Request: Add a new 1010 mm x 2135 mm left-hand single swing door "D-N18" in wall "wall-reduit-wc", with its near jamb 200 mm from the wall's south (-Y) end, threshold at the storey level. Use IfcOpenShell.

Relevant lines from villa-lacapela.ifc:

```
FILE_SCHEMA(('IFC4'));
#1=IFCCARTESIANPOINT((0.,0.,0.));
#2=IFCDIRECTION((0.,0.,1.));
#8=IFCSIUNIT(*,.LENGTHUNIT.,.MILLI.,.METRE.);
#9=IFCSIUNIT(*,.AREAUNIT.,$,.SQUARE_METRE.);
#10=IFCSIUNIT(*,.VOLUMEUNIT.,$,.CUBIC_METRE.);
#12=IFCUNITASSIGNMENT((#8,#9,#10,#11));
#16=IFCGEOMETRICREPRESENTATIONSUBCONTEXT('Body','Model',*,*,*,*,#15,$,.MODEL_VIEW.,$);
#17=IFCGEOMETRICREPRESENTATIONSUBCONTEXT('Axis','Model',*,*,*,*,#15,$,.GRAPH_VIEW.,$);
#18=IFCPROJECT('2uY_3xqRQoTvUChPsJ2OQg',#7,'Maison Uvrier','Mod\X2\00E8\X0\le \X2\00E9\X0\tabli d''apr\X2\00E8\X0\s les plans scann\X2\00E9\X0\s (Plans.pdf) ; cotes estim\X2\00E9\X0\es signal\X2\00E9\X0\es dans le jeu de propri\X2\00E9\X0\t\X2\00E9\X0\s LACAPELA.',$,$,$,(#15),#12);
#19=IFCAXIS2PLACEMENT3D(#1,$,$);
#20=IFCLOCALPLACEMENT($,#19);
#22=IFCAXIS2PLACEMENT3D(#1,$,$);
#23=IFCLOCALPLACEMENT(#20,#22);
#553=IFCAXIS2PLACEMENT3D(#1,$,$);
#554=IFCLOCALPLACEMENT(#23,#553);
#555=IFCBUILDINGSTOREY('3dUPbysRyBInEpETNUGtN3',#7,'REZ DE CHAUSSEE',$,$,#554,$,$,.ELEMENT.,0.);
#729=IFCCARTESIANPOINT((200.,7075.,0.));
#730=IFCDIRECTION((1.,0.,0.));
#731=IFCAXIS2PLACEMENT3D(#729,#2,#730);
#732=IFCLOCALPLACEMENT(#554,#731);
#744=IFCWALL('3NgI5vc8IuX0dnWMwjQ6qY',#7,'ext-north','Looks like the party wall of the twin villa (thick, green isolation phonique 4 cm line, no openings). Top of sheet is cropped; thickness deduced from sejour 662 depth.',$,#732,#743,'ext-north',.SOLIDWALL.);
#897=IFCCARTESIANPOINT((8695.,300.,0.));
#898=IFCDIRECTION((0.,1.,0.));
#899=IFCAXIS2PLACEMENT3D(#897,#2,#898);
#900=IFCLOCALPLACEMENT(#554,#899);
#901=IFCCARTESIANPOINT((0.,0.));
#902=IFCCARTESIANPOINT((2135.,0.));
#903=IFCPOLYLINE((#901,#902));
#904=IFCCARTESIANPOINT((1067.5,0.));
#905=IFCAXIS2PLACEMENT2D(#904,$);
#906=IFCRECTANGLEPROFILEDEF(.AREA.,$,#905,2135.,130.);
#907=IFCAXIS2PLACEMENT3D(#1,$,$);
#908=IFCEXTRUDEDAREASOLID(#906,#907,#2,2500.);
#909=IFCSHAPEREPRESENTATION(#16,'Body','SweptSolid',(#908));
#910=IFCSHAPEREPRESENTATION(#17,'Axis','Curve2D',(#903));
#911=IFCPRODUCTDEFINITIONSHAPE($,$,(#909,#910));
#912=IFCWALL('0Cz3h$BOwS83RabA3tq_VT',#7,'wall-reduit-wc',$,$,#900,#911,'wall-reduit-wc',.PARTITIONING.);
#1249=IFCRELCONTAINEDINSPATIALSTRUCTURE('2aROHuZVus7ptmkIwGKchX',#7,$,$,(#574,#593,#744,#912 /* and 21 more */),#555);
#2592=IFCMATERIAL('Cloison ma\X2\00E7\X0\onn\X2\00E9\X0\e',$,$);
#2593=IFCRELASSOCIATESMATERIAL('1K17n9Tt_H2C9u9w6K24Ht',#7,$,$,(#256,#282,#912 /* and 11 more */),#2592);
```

```python
import numpy as np
import ifcopenshell
import ifcopenshell.api.feature
import ifcopenshell.api.geometry
import ifcopenshell.api.root
import ifcopenshell.api.spatial
import ifcopenshell.geom
import ifcopenshell.util.element
import ifcopenshell.util.placement
import ifcopenshell.util.representation
import ifcopenshell.util.shape
import ifcopenshell.util.unit

model = ifcopenshell.open("villa-lacapela.ifc")
unit_scale = ifcopenshell.util.unit.calculate_unit_scale(model)
settings = ifcopenshell.geom.settings()


def volume(element):
    """Net volume in cubic metres, openings subtracted."""
    shape = ifcopenshell.geom.create_shape(settings, element)
    return ifcopenshell.util.shape.get_volume(shape.geometry)


wall = model.by_id(912)
storey = ifcopenshell.util.element.get_container(wall, ifc_class="IfcBuildingStorey")
context = ifcopenshell.util.representation.get_context(model, "Model", "Body", "MODEL_VIEW")
before = volume(wall)

width, height, from_end, sill = 1.01, 2.135, 0.2, 0.0  # metres

# The wall runs along its own X axis, and the end named is its -X end.
wall_shape = ifcopenshell.geom.create_shape(settings, wall)
x, y, z = ifcopenshell.util.shape.get_vertices(wall_shape.geometry).T
start = x.min() + from_end
face, thickness = float(y.min()), float(y.max() - y.min())
wall_matrix = ifcopenshell.util.placement.get_local_placement(wall.ObjectPlacement)
level = ifcopenshell.util.placement.get_local_placement(storey.ObjectPlacement)[2, 3]


def in_wall(x, y):
    """Placement at x, y metres in the wall's axes, at sill height."""
    matrix = wall_matrix.copy()
    matrix[:, 3] = wall_matrix @ np.array([x / unit_scale, y / unit_scale, 0.0, 1.0])
    matrix[2, 3] = level + sill / unit_scale
    return matrix


# Opening: a box that overshoots both wall faces by 50 mm.
opening = ifcopenshell.api.root.create_entity(model, ifc_class="IfcOpeningElement", predefined_type="OPENING")
box = ifcopenshell.api.geometry.add_wall_representation(
    model, context=context, length=width, height=height, thickness=thickness + 0.1
)
ifcopenshell.api.geometry.assign_representation(model, product=opening, representation=box)
ifcopenshell.api.geometry.edit_object_placement(model, product=opening, matrix=in_wall(start, face - 0.05), is_si=False)
ifcopenshell.api.feature.add_feature(model, feature=opening, element=wall)

door = ifcopenshell.api.root.create_entity(model, ifc_class="IfcDoor", name="D-N18", predefined_type="DOOR")
door.OverallWidth, door.OverallHeight = width / unit_scale, height / unit_scale
door.OperationType = "SINGLE_SWING_LEFT"
body = ifcopenshell.api.geometry.add_door_representation(
    model,
    context=context,
    overall_width=door.OverallWidth,
    overall_height=door.OverallHeight,
    operation_type="SINGLE_SWING_LEFT",
    lining_properties={"LiningDepth": thickness / unit_scale, "ThresholdDepth": thickness / unit_scale},
)
ifcopenshell.api.geometry.assign_representation(model, product=door, representation=body)
ifcopenshell.api.spatial.assign_container(model, products=[door], relating_structure=storey)
ifcopenshell.api.feature.add_filling(model, opening=opening, element=door)

# The lining spans the wall, so the door starts at the wall face.
ifcopenshell.api.geometry.edit_object_placement(model, product=door, matrix=in_wall(start, face), is_si=False)

after = volume(wall)

print(f"wall volume {before:.3f} -> {after:.3f} m3")

model.write("villa-lacapela_rev.ifc")
```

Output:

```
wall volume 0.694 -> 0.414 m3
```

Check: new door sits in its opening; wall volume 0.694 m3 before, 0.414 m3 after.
